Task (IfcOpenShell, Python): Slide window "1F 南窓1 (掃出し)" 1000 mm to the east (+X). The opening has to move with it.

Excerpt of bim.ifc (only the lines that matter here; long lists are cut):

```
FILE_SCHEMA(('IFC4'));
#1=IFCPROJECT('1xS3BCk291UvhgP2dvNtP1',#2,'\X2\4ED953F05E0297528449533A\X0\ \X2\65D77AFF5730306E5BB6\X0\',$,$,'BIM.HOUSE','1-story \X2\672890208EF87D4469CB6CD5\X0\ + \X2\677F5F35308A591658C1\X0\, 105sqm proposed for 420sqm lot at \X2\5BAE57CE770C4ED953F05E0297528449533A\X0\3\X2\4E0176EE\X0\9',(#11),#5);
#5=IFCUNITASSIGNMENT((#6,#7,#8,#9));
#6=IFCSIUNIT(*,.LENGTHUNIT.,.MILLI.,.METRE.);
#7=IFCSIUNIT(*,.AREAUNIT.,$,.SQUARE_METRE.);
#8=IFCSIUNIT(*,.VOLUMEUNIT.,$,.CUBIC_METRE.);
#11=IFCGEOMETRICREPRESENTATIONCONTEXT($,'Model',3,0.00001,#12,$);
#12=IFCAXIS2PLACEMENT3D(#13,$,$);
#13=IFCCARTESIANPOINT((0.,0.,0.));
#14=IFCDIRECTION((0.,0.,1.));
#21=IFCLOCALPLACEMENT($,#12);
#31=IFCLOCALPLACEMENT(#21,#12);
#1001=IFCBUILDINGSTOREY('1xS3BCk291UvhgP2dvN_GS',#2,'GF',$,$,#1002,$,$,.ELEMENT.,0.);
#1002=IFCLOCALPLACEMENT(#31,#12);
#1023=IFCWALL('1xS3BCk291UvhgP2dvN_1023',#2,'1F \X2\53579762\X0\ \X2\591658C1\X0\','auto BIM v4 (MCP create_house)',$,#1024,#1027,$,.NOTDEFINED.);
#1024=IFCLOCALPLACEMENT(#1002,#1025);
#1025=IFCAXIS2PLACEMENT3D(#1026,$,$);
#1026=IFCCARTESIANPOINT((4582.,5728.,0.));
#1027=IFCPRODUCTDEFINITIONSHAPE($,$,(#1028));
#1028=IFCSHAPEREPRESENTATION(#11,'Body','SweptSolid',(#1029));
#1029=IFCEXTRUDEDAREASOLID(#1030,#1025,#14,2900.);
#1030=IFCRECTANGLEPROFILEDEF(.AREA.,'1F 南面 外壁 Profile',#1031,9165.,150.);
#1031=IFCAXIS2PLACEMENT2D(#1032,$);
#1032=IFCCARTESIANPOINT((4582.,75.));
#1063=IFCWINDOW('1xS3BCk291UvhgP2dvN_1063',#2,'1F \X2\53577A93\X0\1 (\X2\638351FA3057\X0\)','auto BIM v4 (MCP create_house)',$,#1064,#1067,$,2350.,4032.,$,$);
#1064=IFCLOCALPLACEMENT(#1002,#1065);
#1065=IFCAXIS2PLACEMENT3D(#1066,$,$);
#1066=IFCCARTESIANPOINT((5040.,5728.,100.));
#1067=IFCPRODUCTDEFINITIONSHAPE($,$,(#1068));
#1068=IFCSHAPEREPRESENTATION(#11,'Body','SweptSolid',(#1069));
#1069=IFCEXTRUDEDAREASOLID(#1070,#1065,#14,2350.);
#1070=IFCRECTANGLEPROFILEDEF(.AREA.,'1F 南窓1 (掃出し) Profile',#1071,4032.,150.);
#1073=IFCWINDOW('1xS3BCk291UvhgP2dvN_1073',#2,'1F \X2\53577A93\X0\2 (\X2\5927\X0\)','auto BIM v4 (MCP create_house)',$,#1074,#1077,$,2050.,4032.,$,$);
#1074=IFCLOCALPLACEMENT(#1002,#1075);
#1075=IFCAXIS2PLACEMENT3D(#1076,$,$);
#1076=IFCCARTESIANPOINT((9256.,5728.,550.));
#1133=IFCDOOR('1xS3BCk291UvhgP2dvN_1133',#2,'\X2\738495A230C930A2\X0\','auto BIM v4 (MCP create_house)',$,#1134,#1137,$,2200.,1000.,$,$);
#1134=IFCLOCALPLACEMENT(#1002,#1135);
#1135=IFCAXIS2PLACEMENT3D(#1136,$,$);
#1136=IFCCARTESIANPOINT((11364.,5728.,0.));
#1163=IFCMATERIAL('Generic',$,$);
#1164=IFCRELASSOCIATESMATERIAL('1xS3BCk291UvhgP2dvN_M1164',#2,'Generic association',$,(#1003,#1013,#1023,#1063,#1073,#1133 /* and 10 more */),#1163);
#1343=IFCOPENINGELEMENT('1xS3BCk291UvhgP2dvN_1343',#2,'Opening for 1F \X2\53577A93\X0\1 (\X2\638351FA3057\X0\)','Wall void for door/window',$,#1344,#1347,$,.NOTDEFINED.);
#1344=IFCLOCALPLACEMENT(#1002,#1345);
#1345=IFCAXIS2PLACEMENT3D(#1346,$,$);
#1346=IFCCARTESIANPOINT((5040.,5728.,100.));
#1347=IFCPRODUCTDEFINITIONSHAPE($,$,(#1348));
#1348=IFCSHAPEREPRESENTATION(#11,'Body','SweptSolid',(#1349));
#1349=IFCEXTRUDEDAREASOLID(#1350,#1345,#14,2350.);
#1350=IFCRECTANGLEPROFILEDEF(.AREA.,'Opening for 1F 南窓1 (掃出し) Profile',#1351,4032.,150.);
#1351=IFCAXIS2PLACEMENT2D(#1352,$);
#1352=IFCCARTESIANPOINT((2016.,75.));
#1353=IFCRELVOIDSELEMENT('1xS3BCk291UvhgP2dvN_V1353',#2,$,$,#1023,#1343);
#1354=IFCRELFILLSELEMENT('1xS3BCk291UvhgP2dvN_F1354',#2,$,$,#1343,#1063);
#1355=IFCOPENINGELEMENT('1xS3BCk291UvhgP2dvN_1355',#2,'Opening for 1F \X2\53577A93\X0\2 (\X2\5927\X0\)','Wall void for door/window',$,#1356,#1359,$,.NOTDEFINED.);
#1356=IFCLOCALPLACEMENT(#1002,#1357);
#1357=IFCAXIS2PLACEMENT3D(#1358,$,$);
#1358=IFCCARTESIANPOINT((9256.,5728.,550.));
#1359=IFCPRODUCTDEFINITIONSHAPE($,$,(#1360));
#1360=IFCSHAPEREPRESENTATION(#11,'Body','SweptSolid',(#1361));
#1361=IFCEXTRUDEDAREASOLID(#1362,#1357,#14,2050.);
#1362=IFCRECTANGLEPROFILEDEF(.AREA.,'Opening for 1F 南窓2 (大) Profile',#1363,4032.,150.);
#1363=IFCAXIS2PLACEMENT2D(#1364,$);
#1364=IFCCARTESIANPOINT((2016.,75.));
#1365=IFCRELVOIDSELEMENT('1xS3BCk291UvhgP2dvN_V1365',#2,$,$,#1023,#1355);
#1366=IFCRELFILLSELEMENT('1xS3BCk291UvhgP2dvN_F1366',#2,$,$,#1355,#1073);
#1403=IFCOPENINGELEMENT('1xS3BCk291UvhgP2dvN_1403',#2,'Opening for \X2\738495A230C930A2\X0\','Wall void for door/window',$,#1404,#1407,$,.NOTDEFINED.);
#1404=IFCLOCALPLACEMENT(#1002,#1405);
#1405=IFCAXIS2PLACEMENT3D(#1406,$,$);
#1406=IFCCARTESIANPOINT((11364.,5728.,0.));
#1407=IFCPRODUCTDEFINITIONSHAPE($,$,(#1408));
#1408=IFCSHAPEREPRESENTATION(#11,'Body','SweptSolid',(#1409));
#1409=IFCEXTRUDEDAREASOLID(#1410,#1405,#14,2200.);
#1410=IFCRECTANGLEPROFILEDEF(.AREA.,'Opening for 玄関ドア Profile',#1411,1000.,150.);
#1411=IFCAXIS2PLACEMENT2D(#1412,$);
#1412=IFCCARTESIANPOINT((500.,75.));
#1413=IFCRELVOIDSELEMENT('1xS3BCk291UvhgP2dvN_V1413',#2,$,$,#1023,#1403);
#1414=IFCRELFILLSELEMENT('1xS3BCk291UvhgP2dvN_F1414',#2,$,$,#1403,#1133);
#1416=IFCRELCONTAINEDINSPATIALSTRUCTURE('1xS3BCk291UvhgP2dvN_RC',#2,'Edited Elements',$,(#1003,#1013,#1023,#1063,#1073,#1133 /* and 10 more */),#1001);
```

```python
import ifcopenshell
import ifcopenshell.api.geometry
import ifcopenshell.util.placement
import ifcopenshell.util.unit

model = ifcopenshell.open("bim.ifc")
unit_scale = ifcopenshell.util.unit.calculate_unit_scale(model)

window = model.by_id(1063)
opening = window.FillsVoids[0].RelatingOpeningElement
wall = opening.VoidsElements[0].RelatingBuildingElement

wall_matrix = ifcopenshell.util.placement.get_local_placement(wall.ObjectPlacement)
shift = wall_matrix[:3, 0] * 1 / unit_scale
before = ifcopenshell.util.placement.get_local_placement(window.ObjectPlacement)[:3, 3].copy()

# The window is not placed relative to its opening, so move both.
for product in (opening, window):
    matrix = ifcopenshell.util.placement.get_local_placement(product.ObjectPlacement)
    matrix[:3, 3] += shift
    ifcopenshell.api.geometry.edit_object_placement(model, product=product, matrix=matrix, is_si=False)

after = ifcopenshell.util.placement.get_local_placement(window.ObjectPlacement)[:3, 3]
print("window moved by", (after - before).round(3) + 0.0)

model.write("bim_rev.ifc")
```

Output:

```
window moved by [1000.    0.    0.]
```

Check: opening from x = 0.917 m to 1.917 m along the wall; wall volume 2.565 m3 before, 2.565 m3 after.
